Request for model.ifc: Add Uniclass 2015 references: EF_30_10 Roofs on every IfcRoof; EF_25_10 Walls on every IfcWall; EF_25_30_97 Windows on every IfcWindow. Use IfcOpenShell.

First a look at what the model holds.

```python
import ifcopenshell

model = ifcopenshell.open("model.ifc")
print(model.schema)
print("classifications:", [c.Name for c in model.by_type("IfcClassification")])
for ifc_class in ("IfcDoor", "IfcRoof", "IfcStair", "IfcWall", "IfcWindow"):
    print(ifc_class, len(model.by_type(ifc_class)))
```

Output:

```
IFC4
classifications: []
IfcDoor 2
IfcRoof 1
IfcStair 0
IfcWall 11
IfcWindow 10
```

```python
import ifcopenshell
import ifcopenshell.api.classification

model = ifcopenshell.open("model.ifc")

system = ifcopenshell.api.classification.add_classification(model, classification="Uniclass 2015")

codes = {
    "IfcRoof": ("EF_30_10", "Roofs"),
    "IfcWall": ("EF_25_10", "Walls"),
    "IfcWindow": ("EF_25_30_97", "Windows"),
}
for ifc_class, (code, name) in codes.items():
    products = model.by_type(ifc_class)
    ifcopenshell.api.classification.add_reference(
        model, products=products, classification=system, identification=code, name=name
    )
    print(code, len(products))

model.write("model_updated.ifc")
```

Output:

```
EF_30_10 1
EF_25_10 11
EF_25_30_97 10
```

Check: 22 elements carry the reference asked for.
